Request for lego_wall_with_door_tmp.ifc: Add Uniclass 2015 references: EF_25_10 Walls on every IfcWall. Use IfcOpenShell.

First a look at what the model holds.

```python
import ifcopenshell

model = ifcopenshell.open("lego_wall_with_door_tmp.ifc")
print(model.schema)
print("classifications:", [c.Name for c in model.by_type("IfcClassification")])
for ifc_class in ("IfcDoor", "IfcRoof", "IfcStair", "IfcWall", "IfcWindow"):
    print(ifc_class, len(model.by_type(ifc_class)))
```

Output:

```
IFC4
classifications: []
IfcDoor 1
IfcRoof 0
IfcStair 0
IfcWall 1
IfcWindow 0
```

```python
import ifcopenshell
import ifcopenshell.api.classification

model = ifcopenshell.open("lego_wall_with_door_tmp.ifc")

system = ifcopenshell.api.classification.add_classification(model, classification="Uniclass 2015")

codes = {
    "IfcWall": ("EF_25_10", "Walls"),
}
for ifc_class, (code, name) in codes.items():
    products = model.by_type(ifc_class)
    ifcopenshell.api.classification.add_reference(
        model, products=products, classification=system, identification=code, name=name
    )
    print(code, len(products))

model.write("lego_wall_with_door_tmp_updated.ifc")
```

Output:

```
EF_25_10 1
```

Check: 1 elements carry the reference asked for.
